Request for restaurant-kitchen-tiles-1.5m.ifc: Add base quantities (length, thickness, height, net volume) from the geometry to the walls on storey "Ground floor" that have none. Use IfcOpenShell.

First a look at what the model holds.

```python
import ifcopenshell
import ifcopenshell.util.element
import ifcopenshell.util.unit

model = ifcopenshell.open("restaurant-kitchen-tiles-1.5m.ifc")
print(model.schema)
for unit_type in ("LENGTHUNIT", "AREAUNIT", "VOLUMEUNIT"):
    print(unit_type, ifcopenshell.util.unit.calculate_unit_scale(model, unit_type))
storey = next(s for s in model.by_type("IfcBuildingStorey") if s.Name == "Ground floor")
walls = [e for e in ifcopenshell.util.element.get_decomposition(storey) if e.is_a("IfcWall")]
for e in sorted(walls, key=lambda e: e.id()):
    print(e.id(), e.is_a(), e.Name, list(ifcopenshell.util.element.get_psets(e, qtos_only=True)), sep=" | ")
```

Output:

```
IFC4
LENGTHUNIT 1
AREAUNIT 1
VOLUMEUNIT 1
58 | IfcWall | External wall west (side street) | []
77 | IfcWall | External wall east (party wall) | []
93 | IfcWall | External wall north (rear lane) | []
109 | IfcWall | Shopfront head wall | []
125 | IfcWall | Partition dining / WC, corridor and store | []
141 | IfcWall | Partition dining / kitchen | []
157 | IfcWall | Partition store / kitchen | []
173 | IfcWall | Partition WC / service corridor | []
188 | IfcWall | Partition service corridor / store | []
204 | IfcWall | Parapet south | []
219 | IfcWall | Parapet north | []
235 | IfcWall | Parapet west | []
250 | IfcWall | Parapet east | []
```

```python
import ifcopenshell
import ifcopenshell.api.pset
import ifcopenshell.geom
import ifcopenshell.util.element
import ifcopenshell.util.shape
import ifcopenshell.util.unit

model = ifcopenshell.open("restaurant-kitchen-tiles-1.5m.ifc")
unit_scale = ifcopenshell.util.unit.calculate_unit_scale(model)
volume_scale = ifcopenshell.util.unit.calculate_unit_scale(model, "VOLUMEUNIT")
settings = ifcopenshell.geom.settings()

storey = next(s for s in model.by_type("IfcBuildingStorey") if s.Name == "Ground floor")
walls = [e for e in ifcopenshell.util.element.get_decomposition(storey) if e.is_a("IfcWall")]

for e in sorted(walls, key=lambda e: e.id()):
    if ifcopenshell.util.element.get_psets(e, qtos_only=True, should_inherit=False):
        continue
    # Geometry comes back in metres, in the element's own axes.
    shape = ifcopenshell.geom.create_shape(settings, e)
    values = {
        "Length": ifcopenshell.util.shape.get_x(shape.geometry) / unit_scale,
        "Width": ifcopenshell.util.shape.get_y(shape.geometry) / unit_scale,
        "Height": ifcopenshell.util.shape.get_z(shape.geometry) / unit_scale,
        "NetVolume": ifcopenshell.util.shape.get_volume(shape.geometry) / volume_scale,
    }
    qto = ifcopenshell.api.pset.add_qto(model, product=e, name="Qto_WallBaseQuantities")
    ifcopenshell.api.pset.edit_qto(model, qto=qto, properties=values)
    print(e.id(), {k: round(v, 3) for k, v in values.items()})

model.write("restaurant-kitchen-tiles-1.5m-out.ifc")
```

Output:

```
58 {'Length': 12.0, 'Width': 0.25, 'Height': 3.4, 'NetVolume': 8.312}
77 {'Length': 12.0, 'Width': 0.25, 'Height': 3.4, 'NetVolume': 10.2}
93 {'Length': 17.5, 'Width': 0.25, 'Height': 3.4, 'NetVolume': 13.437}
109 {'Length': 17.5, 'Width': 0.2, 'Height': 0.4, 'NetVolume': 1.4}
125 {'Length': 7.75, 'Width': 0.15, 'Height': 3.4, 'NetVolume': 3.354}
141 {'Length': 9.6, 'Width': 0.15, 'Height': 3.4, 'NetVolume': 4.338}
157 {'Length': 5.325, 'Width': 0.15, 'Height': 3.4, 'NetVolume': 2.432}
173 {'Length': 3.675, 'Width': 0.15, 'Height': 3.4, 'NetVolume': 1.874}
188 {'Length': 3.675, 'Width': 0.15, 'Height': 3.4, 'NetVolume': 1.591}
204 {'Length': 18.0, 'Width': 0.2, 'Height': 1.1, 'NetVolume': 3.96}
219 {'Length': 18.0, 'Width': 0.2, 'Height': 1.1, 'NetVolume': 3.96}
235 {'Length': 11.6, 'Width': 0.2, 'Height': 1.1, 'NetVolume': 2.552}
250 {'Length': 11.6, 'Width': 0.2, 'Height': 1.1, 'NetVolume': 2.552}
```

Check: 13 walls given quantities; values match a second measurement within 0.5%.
